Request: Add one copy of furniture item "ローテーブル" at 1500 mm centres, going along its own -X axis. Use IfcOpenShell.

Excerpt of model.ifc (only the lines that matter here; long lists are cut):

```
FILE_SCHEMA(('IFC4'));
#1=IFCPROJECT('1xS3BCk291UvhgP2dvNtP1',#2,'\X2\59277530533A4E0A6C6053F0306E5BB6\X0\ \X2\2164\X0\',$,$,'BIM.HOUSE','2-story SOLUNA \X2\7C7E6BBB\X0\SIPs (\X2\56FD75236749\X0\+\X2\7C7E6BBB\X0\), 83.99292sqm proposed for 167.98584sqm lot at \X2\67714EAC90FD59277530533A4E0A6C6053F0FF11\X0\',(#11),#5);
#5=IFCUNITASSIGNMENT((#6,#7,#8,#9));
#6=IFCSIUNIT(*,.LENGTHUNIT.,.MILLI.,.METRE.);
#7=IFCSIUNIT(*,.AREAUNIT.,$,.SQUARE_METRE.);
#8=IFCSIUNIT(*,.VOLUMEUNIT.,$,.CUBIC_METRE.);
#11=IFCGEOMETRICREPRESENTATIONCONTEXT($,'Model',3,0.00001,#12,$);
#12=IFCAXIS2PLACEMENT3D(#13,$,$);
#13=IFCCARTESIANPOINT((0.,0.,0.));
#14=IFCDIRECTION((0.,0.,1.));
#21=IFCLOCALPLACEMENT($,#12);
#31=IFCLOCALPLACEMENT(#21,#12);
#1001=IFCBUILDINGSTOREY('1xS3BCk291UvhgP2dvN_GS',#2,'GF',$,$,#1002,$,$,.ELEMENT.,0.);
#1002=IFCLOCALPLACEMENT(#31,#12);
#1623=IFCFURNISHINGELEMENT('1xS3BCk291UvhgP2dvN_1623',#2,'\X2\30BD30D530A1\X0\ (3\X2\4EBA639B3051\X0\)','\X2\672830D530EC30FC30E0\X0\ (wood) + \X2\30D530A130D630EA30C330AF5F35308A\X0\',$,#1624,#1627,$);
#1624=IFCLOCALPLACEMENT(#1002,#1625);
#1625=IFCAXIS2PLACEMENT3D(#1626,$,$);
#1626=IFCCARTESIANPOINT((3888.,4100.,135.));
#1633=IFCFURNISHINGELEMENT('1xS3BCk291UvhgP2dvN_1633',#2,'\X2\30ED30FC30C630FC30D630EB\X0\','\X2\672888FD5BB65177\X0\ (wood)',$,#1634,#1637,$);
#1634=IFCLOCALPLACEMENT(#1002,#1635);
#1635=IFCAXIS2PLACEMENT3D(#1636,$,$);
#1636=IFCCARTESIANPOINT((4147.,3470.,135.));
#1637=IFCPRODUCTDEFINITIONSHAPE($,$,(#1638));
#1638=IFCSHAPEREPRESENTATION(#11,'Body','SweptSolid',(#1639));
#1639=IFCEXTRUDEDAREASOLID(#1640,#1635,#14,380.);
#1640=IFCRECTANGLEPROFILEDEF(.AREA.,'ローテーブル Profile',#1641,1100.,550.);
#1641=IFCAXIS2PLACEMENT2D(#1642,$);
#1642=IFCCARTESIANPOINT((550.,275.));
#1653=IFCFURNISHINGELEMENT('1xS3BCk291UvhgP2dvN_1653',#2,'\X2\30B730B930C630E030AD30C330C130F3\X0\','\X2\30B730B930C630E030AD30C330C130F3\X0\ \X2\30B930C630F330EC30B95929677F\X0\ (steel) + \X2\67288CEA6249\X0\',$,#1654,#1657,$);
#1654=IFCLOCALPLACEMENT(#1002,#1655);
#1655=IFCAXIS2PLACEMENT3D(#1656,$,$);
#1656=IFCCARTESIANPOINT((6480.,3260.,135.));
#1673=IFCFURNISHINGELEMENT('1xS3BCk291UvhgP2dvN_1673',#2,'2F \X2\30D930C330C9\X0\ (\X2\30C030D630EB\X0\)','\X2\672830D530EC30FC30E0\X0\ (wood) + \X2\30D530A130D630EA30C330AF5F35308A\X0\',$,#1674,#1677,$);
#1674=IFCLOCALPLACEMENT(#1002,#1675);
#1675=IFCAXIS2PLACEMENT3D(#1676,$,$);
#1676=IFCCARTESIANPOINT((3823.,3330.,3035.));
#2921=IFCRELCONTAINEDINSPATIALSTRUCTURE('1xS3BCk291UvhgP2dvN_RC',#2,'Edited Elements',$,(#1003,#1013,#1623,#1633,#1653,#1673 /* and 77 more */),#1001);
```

```python
import ifcopenshell
import ifcopenshell.api.geometry
import ifcopenshell.api.root
import ifcopenshell.util.element
import ifcopenshell.util.placement

model = ifcopenshell.open("model.ifc")


def reuse_history(source, copy):
    """copy_class also copies each property set's owner history, people and application; keep the originals."""
    for rel in copy.IsDefinedBy:
        if rel.is_a("IfcRelDefinesByProperties") and (history := rel.RelatingPropertyDefinition.OwnerHistory):
            rel.RelatingPropertyDefinition.OwnerHistory = source.OwnerHistory
            ifcopenshell.util.element.remove_deep2(model, history)


source = model.by_guid("1xS3BCk291UvhgP2dvN_1633")
base = ifcopenshell.util.placement.get_local_placement(source.ObjectPlacement)
step = -base[:3, 0] * 1500.0

for i in range(1, 2):
    copy = ifcopenshell.api.root.copy_class(model, product=source)
    copy.Representation = ifcopenshell.util.element.copy_deep(
        model, source.Representation, exclude=["IfcGeometricRepresentationContext", "IfcRepresentationMap"]
    )
    reuse_history(source, copy)
    matrix = base.copy()
    matrix[:3, 3] += i * step
    print("added at", matrix[:3, 3].round(3) + 0.0)
    ifcopenshell.api.geometry.edit_object_placement(model, product=copy, matrix=matrix, is_si=False)

model.write("model-out.ifc")
```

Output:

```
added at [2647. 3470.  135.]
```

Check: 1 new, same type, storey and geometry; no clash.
